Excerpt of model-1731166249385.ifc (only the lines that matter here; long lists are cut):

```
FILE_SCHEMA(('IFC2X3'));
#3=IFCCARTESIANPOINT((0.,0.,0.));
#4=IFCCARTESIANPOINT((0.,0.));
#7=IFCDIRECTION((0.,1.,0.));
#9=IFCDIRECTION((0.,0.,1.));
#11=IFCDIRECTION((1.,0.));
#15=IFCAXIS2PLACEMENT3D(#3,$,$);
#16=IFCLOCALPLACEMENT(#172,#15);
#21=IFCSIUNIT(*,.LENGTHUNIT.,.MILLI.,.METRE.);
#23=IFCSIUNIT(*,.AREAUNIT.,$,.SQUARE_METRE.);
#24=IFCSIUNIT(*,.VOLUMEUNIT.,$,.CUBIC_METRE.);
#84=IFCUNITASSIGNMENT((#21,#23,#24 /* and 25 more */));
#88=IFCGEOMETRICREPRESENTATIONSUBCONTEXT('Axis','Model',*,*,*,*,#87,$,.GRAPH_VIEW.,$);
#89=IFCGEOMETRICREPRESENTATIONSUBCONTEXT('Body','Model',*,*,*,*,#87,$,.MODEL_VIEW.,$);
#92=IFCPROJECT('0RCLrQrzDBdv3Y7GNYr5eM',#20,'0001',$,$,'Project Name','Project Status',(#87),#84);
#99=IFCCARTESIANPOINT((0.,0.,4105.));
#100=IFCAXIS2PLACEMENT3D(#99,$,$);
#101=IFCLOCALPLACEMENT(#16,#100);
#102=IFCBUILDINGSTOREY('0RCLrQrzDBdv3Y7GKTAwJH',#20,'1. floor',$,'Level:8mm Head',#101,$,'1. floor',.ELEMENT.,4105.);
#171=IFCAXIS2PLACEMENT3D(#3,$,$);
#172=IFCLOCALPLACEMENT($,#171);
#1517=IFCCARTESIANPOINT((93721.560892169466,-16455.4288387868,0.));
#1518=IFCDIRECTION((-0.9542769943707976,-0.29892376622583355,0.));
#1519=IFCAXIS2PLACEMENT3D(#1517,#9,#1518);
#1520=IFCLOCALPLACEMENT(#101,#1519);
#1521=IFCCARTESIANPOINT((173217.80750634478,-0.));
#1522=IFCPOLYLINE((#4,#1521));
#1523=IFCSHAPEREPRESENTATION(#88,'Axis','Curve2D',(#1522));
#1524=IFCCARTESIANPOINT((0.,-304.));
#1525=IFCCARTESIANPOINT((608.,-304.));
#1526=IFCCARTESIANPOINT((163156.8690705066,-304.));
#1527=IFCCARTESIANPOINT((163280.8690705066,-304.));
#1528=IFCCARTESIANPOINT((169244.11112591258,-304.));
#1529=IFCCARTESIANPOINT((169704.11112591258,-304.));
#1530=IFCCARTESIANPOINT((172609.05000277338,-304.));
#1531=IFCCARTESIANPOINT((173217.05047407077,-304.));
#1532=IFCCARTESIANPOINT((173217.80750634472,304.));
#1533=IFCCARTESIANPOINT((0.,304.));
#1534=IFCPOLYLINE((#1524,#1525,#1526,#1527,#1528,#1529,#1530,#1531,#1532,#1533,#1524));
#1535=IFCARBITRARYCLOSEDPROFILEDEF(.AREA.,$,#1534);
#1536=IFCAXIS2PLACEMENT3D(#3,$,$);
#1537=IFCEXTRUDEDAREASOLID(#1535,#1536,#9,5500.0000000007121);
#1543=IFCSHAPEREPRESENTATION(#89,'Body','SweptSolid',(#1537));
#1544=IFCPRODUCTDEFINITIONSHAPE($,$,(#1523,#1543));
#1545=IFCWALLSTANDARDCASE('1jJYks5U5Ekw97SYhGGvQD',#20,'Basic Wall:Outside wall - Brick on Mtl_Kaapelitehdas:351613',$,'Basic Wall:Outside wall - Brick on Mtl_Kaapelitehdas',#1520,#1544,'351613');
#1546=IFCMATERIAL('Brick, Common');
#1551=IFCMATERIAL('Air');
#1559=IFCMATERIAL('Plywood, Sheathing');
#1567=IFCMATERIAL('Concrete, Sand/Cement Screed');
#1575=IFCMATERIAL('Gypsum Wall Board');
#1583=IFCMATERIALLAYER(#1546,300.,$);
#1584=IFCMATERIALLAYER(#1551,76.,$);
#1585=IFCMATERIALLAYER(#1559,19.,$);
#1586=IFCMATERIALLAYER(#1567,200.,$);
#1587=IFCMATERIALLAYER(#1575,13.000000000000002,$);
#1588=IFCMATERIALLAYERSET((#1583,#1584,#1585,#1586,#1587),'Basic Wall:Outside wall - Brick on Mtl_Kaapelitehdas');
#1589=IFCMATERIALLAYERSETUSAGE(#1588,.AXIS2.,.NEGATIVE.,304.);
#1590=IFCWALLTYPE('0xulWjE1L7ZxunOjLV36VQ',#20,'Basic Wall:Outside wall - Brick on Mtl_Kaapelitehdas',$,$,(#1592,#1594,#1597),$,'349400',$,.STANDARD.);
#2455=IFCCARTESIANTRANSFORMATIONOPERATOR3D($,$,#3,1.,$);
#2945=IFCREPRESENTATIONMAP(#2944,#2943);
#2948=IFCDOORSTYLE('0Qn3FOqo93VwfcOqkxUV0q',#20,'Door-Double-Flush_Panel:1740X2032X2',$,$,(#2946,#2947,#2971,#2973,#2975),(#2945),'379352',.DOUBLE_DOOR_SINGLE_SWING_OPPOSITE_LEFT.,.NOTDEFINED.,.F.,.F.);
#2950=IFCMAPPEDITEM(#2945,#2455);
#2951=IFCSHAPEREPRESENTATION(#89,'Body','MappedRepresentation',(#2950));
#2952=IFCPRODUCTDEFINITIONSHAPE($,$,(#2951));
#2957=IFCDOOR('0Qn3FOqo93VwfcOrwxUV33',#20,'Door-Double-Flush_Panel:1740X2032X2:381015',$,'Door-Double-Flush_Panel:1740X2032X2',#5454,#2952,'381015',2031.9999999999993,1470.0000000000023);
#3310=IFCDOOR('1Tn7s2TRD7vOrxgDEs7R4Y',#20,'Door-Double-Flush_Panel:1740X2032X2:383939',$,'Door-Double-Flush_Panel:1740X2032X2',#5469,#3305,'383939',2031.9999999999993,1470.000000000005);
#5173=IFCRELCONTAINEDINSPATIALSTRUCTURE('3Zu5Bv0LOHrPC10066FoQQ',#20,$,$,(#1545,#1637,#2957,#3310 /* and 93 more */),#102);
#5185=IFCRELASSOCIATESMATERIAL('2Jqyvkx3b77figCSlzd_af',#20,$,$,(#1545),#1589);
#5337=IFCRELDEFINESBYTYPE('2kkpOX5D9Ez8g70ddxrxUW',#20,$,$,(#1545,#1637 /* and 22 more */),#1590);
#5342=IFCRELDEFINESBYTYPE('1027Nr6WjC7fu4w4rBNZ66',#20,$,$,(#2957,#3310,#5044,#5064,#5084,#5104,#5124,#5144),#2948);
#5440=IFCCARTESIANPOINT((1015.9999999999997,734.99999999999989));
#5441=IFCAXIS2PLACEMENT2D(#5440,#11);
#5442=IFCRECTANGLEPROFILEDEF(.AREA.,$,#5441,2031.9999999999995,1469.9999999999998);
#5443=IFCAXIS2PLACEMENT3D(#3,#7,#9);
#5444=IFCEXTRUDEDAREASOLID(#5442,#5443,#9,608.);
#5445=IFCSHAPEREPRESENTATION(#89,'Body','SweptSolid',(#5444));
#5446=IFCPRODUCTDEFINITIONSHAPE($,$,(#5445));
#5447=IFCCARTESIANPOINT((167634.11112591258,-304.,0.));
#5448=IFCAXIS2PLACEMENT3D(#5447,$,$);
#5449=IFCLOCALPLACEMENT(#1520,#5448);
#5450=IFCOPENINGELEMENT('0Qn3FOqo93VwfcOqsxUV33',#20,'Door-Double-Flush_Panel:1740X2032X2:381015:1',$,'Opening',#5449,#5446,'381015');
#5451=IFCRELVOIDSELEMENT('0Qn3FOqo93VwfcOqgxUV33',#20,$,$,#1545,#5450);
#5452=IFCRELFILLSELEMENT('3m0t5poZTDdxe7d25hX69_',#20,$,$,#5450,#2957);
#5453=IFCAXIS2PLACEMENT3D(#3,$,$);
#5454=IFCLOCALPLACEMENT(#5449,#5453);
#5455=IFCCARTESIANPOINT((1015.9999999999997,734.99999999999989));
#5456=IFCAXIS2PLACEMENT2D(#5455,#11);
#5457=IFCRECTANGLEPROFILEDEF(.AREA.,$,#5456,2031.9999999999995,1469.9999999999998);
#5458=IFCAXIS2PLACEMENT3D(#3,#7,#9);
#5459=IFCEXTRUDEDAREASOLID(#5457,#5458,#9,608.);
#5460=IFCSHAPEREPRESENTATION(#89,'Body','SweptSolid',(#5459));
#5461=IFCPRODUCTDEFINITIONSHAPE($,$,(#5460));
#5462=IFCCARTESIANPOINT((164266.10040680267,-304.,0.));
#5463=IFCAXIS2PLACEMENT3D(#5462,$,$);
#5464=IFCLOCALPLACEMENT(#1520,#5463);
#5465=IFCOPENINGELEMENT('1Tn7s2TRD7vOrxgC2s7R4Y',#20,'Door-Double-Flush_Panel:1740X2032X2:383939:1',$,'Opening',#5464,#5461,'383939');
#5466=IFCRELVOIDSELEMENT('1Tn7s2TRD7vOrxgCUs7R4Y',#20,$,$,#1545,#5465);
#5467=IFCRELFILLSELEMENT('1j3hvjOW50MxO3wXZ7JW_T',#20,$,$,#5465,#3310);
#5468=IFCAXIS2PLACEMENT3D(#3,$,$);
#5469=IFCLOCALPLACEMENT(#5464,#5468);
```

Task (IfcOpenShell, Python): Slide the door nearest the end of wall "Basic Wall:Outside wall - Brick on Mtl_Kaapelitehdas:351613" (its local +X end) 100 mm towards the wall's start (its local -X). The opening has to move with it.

```python
import ifcopenshell
import ifcopenshell.api.geometry
import ifcopenshell.util.placement
import ifcopenshell.util.unit

model = ifcopenshell.open("model-1731166249385.ifc")
unit_scale = ifcopenshell.util.unit.calculate_unit_scale(model)

door = model.by_guid("0Qn3FOqo93VwfcOrwxUV33")
opening = door.FillsVoids[0].RelatingOpeningElement
wall = opening.VoidsElements[0].RelatingBuildingElement

wall_matrix = ifcopenshell.util.placement.get_local_placement(wall.ObjectPlacement)
shift = wall_matrix[:3, 0] * -0.1 / unit_scale
before = ifcopenshell.util.placement.get_local_placement(door.ObjectPlacement)[:3, 3].copy()

# The door is placed relative to its opening, so it follows when the opening moves.
matrix = ifcopenshell.util.placement.get_local_placement(opening.ObjectPlacement)
matrix[:3, 3] += shift
ifcopenshell.api.geometry.edit_object_placement(
    model, product=opening, matrix=matrix, is_si=False, should_transform_children=True
)

after = ifcopenshell.util.placement.get_local_placement(door.ObjectPlacement)[:3, 3]
print("door moved by", (after - before).round(3) + 0.0)

model.write("model-1731166249385_v2.ifc")
```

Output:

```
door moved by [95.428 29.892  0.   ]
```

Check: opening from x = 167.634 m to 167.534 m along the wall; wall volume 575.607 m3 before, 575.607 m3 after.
